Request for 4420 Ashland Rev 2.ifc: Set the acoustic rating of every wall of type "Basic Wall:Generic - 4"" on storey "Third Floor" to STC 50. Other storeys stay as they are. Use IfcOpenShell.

First a look at what the model holds.

```python
import ifcopenshell
import ifcopenshell.util.element

model = ifcopenshell.open("4420 Ashland Rev 2.ifc")
print(model.schema)
storey = next(s for s in model.by_type("IfcBuildingStorey") if s.Name == "Third Floor")
walls = [e for e in ifcopenshell.util.element.get_decomposition(storey) if e.is_a("IfcWall")]
seen = {}
for e in walls:
    element_type = ifcopenshell.util.element.get_type(e)
    key = (element_type.Name if element_type != e and element_type else None, ifcopenshell.util.element.get_pset(e, "Pset_WallCommon", "AcousticRating"))
    seen[key] = seen.get(key, 0) + 1
for (name, value), count in sorted(seen.items(), key=str):
    print(count, "x", name, "|", value)
```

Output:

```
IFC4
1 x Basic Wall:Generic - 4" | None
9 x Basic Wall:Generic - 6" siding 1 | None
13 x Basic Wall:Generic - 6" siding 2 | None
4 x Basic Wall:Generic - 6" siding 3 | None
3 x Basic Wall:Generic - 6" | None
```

```python
import ifcopenshell
import ifcopenshell.api.pset
import ifcopenshell.util.element

model = ifcopenshell.open("4420 Ashland Rev 2.ifc")

storey = next(s for s in model.by_type("IfcBuildingStorey") if s.Name == "Third Floor")
walls = [e for e in ifcopenshell.util.element.get_decomposition(storey) if e.is_a("IfcWall")]

count = 0
for e in walls:
    element_type = ifcopenshell.util.element.get_type(e)
    if element_type in (None, e) or element_type.Name != 'Basic Wall:Generic - 4"':
        continue
    # add_pset returns the element's existing set when there is one.
    pset = ifcopenshell.api.pset.add_pset(model, product=e, name="Pset_WallCommon")
    ifcopenshell.api.pset.edit_pset(model, pset=pset, properties={"AcousticRating": "STC 50"})
    count += 1

print(count, "walls updated")

model.write("4420 Ashland Rev 2_rev.ifc")
```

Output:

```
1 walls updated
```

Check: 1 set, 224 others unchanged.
